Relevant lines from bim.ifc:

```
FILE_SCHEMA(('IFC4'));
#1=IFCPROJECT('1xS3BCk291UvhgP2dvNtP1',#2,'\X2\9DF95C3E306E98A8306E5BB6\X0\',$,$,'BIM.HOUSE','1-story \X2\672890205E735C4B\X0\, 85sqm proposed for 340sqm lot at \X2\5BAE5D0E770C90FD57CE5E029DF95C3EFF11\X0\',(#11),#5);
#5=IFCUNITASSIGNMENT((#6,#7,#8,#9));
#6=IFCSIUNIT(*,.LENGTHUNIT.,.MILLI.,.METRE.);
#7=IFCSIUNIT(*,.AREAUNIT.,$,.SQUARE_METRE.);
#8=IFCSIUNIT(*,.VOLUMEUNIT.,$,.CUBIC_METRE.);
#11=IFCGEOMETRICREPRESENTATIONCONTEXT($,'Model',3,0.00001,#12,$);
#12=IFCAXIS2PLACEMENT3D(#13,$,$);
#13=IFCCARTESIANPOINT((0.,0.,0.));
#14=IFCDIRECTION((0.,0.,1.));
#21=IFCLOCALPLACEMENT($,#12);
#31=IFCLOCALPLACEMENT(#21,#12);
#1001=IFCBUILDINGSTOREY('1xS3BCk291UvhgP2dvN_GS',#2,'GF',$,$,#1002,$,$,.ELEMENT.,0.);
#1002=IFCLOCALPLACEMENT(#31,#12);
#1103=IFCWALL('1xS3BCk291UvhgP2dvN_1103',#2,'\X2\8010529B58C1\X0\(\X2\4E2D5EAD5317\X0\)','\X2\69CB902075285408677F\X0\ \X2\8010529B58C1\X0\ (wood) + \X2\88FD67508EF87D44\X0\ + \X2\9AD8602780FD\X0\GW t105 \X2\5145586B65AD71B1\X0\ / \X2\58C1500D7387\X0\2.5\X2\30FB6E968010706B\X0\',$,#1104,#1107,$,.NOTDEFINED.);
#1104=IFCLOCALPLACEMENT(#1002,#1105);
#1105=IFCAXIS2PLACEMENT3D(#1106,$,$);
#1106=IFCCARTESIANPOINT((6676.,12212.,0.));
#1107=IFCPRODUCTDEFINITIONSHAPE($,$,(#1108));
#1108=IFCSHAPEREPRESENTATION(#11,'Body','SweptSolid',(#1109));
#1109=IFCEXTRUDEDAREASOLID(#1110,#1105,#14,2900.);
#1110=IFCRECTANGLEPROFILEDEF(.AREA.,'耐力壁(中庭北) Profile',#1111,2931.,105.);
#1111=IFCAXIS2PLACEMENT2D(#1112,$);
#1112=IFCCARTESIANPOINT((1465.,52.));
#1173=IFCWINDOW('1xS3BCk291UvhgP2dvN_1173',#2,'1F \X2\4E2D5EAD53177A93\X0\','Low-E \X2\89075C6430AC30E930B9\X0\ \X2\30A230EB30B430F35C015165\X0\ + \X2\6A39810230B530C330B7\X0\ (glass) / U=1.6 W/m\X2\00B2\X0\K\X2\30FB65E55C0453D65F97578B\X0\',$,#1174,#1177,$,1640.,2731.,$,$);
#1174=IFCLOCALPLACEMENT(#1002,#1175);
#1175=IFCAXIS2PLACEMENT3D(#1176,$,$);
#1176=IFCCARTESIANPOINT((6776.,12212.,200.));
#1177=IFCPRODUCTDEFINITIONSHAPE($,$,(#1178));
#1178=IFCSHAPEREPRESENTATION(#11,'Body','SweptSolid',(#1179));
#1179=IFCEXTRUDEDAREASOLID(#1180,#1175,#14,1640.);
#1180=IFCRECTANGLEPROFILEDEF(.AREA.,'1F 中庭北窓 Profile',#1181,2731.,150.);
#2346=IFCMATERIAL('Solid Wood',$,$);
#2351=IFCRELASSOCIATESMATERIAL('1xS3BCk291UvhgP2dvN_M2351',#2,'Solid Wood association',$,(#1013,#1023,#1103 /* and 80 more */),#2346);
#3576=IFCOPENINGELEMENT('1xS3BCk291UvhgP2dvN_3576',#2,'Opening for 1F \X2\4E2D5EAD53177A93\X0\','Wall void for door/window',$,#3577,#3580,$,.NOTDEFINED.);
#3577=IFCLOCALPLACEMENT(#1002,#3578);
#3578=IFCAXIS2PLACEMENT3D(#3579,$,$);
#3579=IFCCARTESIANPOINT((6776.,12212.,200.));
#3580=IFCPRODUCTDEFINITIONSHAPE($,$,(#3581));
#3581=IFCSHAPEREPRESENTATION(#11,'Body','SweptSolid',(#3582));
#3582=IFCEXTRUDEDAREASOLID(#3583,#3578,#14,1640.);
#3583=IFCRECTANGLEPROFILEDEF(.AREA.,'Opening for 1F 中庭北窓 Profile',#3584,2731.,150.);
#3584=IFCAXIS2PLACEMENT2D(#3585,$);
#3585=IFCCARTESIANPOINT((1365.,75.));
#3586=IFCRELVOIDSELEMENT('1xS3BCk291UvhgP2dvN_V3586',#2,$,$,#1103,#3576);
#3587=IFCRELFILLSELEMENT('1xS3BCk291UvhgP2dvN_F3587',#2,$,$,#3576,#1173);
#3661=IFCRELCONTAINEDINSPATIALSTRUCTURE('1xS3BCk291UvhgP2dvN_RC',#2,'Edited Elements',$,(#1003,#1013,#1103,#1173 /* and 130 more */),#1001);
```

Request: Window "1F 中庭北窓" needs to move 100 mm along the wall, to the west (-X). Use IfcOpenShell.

```python
import ifcopenshell
import ifcopenshell.api.geometry
import ifcopenshell.util.placement

model = ifcopenshell.open("bim.ifc")

window = model.by_guid("1xS3BCk291UvhgP2dvN_1173")
opening = window.FillsVoids[0].RelatingOpeningElement
wall = opening.VoidsElements[0].RelatingBuildingElement

wall_matrix = ifcopenshell.util.placement.get_local_placement(wall.ObjectPlacement)
shift = wall_matrix[:3, 0] * -100.0
before = ifcopenshell.util.placement.get_local_placement(window.ObjectPlacement)[:3, 3].copy()

# The window is not placed relative to its opening, so move both.
for product in (opening, window):
    matrix = ifcopenshell.util.placement.get_local_placement(product.ObjectPlacement)
    matrix[:3, 3] += shift
    ifcopenshell.api.geometry.edit_object_placement(model, product=product, matrix=matrix, is_si=False)

after = ifcopenshell.util.placement.get_local_placement(window.ObjectPlacement)[:3, 3]
print("window moved by", (after - before).round(3) + 0.0)

model.write("bim_edited.ifc")
```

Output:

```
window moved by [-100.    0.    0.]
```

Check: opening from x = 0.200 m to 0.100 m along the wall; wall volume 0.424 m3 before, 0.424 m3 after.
